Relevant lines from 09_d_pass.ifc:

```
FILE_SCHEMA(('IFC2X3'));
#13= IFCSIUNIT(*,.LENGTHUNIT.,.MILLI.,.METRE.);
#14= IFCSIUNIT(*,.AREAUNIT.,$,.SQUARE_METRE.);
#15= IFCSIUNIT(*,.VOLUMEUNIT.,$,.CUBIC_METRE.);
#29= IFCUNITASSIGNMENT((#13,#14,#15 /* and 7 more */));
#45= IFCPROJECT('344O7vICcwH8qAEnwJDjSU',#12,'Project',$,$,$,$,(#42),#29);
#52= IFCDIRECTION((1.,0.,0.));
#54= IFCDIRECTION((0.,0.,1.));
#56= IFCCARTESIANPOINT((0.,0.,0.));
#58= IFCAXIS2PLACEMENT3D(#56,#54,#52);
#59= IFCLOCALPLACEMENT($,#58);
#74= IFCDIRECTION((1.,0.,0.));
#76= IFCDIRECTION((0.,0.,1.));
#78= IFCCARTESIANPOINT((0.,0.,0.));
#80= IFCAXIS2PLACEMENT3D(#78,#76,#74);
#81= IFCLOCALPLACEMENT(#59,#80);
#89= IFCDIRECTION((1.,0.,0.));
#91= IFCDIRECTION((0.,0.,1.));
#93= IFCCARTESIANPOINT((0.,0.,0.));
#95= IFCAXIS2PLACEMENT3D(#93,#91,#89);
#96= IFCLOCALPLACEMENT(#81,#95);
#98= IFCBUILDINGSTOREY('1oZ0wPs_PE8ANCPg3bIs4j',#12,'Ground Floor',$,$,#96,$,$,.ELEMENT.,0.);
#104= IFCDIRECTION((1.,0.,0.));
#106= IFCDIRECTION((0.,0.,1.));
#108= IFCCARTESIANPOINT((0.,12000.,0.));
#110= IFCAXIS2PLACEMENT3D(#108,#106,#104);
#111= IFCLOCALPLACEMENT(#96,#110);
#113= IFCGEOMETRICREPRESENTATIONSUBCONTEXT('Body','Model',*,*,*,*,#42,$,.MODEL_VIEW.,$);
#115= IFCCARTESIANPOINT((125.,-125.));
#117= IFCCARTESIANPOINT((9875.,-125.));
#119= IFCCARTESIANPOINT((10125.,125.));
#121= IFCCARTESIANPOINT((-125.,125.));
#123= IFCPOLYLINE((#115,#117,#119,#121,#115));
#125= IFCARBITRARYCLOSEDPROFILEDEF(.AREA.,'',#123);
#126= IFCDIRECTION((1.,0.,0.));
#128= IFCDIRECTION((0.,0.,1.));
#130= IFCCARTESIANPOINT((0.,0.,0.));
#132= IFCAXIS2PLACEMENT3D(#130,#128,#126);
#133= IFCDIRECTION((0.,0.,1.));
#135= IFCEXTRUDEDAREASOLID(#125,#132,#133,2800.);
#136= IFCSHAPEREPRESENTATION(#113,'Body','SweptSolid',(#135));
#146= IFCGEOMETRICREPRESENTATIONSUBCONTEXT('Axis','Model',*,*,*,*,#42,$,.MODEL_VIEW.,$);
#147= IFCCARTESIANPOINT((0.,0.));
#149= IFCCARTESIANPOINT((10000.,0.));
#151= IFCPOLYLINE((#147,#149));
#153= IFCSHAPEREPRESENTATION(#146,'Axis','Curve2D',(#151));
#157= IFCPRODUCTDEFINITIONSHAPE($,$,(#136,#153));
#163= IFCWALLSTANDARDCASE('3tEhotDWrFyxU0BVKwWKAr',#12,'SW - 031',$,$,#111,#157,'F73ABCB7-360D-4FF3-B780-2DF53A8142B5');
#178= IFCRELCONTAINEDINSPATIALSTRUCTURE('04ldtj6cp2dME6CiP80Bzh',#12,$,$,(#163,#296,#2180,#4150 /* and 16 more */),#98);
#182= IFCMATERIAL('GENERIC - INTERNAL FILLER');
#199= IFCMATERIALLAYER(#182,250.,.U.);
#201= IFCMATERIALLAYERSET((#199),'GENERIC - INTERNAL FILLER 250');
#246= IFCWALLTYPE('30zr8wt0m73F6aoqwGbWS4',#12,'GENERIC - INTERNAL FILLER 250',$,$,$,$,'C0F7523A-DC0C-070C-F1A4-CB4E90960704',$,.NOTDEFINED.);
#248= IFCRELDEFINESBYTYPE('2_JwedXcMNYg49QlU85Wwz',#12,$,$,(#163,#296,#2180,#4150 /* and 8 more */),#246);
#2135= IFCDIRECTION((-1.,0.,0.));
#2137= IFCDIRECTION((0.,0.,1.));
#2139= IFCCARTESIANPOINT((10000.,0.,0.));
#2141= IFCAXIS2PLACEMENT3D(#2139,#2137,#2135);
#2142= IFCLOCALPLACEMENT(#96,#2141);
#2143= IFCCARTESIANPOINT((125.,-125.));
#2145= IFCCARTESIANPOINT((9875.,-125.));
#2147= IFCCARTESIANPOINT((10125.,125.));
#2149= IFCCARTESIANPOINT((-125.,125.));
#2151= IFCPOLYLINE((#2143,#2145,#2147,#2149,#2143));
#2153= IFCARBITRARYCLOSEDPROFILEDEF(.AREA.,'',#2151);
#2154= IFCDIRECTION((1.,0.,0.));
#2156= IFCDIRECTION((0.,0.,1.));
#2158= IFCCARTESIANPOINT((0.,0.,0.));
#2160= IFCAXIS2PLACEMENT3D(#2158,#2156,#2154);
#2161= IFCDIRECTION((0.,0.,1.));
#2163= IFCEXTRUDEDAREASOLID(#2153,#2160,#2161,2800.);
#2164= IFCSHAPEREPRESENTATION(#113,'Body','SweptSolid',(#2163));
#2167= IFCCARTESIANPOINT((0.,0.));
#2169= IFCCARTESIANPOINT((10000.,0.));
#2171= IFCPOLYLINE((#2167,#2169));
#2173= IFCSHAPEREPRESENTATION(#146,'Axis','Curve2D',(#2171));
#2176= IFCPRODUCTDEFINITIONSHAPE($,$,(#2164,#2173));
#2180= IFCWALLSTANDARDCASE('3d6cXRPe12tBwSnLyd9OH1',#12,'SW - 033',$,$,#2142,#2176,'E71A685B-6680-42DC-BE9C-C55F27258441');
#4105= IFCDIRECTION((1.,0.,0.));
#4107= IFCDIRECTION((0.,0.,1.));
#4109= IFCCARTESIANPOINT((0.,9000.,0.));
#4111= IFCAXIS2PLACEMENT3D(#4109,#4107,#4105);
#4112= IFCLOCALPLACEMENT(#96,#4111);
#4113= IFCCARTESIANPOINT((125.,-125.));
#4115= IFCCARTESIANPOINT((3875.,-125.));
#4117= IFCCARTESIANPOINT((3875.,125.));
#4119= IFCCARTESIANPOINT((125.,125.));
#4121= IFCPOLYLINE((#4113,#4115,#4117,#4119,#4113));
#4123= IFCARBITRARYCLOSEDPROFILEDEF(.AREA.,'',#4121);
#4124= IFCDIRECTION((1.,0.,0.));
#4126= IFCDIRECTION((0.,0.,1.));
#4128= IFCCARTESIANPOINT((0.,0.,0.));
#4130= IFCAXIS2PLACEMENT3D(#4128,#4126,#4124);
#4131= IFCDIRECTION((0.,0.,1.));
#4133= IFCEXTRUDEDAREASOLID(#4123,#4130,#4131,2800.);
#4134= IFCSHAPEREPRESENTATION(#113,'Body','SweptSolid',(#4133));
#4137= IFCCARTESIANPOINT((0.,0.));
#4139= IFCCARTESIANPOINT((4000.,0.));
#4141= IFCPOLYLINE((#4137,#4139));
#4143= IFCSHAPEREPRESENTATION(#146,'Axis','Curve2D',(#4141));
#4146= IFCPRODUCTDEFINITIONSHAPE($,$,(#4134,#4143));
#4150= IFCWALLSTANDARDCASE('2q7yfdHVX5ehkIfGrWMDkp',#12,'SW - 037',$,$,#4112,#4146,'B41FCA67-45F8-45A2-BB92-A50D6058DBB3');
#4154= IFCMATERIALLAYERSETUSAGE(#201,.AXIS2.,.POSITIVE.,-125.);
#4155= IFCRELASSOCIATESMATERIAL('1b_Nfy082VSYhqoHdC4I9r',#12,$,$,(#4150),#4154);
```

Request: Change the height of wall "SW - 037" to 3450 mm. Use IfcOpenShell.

```python
import ifcopenshell
import ifcopenshell.geom
import ifcopenshell.util.representation
import ifcopenshell.util.shape
import ifcopenshell.util.unit

model = ifcopenshell.open("09_d_pass.ifc")
unit_scale = ifcopenshell.util.unit.calculate_unit_scale(model)
settings = ifcopenshell.geom.settings()


def volume(element):
    """Net volume in cubic metres, openings subtracted."""
    shape = ifcopenshell.geom.create_shape(settings, element)
    return ifcopenshell.util.shape.get_volume(shape.geometry)


wall = model.by_guid("2q7yfdHVX5ehkIfGrWMDkp")
before = volume(wall)

body = ifcopenshell.util.representation.get_representation(wall, "Model", "Body")
solid = body.Items[0]
old_height = solid.Depth
solid.Depth = 3.45 / unit_scale
after = volume(wall)

print(f"height {old_height:g} -> {solid.Depth:g}, volume {before:.3f} -> {after:.3f} m3")

model.write("09_d_pass_edited.ifc")
```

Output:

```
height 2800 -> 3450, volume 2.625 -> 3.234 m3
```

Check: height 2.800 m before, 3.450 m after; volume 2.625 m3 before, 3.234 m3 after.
